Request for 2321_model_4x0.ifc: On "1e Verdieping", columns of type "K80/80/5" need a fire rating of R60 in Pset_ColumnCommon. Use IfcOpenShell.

First a look at what the model holds.

```python
import ifcopenshell
import ifcopenshell.util.element

model = ifcopenshell.open("2321_model_4x0.ifc")
print(model.schema)
storey = next(s for s in model.by_type("IfcBuildingStorey") if s.Name == "1e Verdieping")
columns = [e for e in ifcopenshell.util.element.get_decomposition(storey) if e.is_a("IfcColumn")]
seen = {}
for e in columns:
    element_type = ifcopenshell.util.element.get_type(e)
    key = (element_type.Name if element_type != e and element_type else None, ifcopenshell.util.element.get_pset(e, "Pset_ColumnCommon", "FireRating"))
    seen[key] = seen.get(key, 0) + 1
for (name, value), count in sorted(seen.items(), key=str):
    print(count, "x", name, "|", value)
```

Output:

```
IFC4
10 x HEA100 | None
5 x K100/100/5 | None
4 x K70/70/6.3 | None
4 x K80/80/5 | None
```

```python
import ifcopenshell
import ifcopenshell.api.pset
import ifcopenshell.util.element

model = ifcopenshell.open("2321_model_4x0.ifc")

storey = next(s for s in model.by_type("IfcBuildingStorey") if s.Name == "1e Verdieping")
columns = [e for e in ifcopenshell.util.element.get_decomposition(storey) if e.is_a("IfcColumn")]

count = 0
for e in columns:
    element_type = ifcopenshell.util.element.get_type(e)
    if element_type in (None, e) or element_type.Name != "K80/80/5":
        continue
    # add_pset returns the element's existing set when there is one.
    pset = ifcopenshell.api.pset.add_pset(model, product=e, name="Pset_ColumnCommon")
    ifcopenshell.api.pset.edit_pset(model, pset=pset, properties={"FireRating": "R60"})
    count += 1

print(count, "columns updated")

model.write("2321_model_4x0_updated.ifc")
```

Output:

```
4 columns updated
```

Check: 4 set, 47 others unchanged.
